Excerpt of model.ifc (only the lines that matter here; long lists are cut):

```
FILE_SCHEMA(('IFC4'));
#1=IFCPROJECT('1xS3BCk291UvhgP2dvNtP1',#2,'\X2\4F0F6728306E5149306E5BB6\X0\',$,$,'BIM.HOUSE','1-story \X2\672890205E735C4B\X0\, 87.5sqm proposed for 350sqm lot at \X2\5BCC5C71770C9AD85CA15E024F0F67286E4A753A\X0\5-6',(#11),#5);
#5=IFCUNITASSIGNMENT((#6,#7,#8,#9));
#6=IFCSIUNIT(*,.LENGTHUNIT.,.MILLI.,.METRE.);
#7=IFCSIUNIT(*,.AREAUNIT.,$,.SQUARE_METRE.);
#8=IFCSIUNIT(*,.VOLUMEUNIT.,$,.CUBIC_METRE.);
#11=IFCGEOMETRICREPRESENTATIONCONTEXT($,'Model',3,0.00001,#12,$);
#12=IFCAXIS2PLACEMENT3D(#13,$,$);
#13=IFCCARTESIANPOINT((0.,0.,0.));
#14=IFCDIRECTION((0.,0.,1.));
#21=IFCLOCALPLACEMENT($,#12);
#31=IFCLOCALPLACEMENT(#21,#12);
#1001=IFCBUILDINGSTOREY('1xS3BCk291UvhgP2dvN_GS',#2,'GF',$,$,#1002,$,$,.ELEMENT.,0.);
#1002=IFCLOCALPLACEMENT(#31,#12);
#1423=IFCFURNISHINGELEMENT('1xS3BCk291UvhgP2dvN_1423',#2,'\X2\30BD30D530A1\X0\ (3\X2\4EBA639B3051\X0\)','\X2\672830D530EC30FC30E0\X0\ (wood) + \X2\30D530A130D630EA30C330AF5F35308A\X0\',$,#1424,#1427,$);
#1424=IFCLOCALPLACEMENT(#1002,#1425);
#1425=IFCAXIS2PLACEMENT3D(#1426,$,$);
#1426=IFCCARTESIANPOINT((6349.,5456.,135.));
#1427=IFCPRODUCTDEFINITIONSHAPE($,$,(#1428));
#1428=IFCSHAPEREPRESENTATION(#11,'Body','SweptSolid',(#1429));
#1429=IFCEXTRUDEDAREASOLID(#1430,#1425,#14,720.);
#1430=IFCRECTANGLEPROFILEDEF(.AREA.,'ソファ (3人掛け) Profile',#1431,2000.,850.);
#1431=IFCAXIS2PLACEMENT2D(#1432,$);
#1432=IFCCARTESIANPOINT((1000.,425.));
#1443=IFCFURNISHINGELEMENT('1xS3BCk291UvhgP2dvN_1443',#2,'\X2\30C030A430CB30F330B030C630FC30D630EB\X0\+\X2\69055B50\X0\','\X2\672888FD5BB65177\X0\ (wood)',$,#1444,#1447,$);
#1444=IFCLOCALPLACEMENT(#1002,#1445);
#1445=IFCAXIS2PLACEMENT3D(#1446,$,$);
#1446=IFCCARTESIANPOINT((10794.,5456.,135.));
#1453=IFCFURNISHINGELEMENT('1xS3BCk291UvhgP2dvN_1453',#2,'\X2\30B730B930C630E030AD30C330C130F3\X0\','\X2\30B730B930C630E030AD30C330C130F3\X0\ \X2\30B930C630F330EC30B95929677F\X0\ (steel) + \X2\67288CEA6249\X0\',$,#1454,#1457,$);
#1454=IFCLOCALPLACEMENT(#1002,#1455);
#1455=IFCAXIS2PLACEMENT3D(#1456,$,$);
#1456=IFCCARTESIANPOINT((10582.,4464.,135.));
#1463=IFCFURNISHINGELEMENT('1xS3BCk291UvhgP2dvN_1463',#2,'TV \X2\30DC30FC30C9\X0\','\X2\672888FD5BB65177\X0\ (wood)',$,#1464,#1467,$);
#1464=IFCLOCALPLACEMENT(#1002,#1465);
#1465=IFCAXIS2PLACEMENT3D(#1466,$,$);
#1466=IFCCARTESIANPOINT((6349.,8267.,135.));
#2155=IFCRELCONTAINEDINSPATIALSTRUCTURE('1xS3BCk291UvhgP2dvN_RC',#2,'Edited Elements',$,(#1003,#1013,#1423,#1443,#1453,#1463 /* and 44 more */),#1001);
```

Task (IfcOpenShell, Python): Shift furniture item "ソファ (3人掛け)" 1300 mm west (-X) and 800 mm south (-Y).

```python
import ifcopenshell
import ifcopenshell.api.geometry
import ifcopenshell.util.placement
import ifcopenshell.util.unit

model = ifcopenshell.open("model.ifc")
unit_scale = ifcopenshell.util.unit.calculate_unit_scale(model)

item = model.by_guid("1xS3BCk291UvhgP2dvN_1423")
matrix = ifcopenshell.util.placement.get_local_placement(item.ObjectPlacement)
matrix[0, 3] -= 1.3 / unit_scale
matrix[1, 3] -= 0.8 / unit_scale
ifcopenshell.api.geometry.edit_object_placement(model, product=item, matrix=matrix, is_si=False)

print(ifcopenshell.util.placement.get_local_placement(item.ObjectPlacement).round(3) + 0.0)

model.write("model_edited.ifc")
```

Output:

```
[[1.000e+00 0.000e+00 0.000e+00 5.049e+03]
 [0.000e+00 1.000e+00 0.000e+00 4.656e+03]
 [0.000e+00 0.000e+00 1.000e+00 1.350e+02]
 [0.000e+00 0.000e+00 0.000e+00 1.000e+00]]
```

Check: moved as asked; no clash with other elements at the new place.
